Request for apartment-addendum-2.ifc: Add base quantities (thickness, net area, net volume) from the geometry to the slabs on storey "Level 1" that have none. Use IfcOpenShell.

First a look at what the model holds.

```python
import ifcopenshell
import ifcopenshell.util.element
import ifcopenshell.util.unit

model = ifcopenshell.open("apartment-addendum-2.ifc")
print(model.schema)
for unit_type in ("LENGTHUNIT", "AREAUNIT", "VOLUMEUNIT"):
    print(unit_type, ifcopenshell.util.unit.calculate_unit_scale(model, unit_type))
storey = next(s for s in model.by_type("IfcBuildingStorey") if s.Name == "Level 1")
slabs = [e for e in ifcopenshell.util.element.get_decomposition(storey) if e.is_a("IfcSlab")]
for e in sorted(slabs, key=lambda e: e.id()):
    print(e.id(), e.is_a(), e.Name, list(ifcopenshell.util.element.get_psets(e, qtos_only=True)), sep=" | ")
```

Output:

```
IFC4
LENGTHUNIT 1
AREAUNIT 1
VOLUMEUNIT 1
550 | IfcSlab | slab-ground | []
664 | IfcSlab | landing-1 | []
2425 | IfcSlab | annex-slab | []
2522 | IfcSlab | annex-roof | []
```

```python
import ifcopenshell
import ifcopenshell.api.pset
import ifcopenshell.geom
import ifcopenshell.util.element
import ifcopenshell.util.shape
import ifcopenshell.util.unit

model = ifcopenshell.open("apartment-addendum-2.ifc")
unit_scale = ifcopenshell.util.unit.calculate_unit_scale(model)
area_scale = ifcopenshell.util.unit.calculate_unit_scale(model, "AREAUNIT")
volume_scale = ifcopenshell.util.unit.calculate_unit_scale(model, "VOLUMEUNIT")
settings = ifcopenshell.geom.settings()

storey = next(s for s in model.by_type("IfcBuildingStorey") if s.Name == "Level 1")
slabs = [e for e in ifcopenshell.util.element.get_decomposition(storey) if e.is_a("IfcSlab")]

for e in sorted(slabs, key=lambda e: e.id()):
    if ifcopenshell.util.element.get_psets(e, qtos_only=True, should_inherit=False):
        continue
    # Geometry comes back in metres, in the element's own axes.
    shape = ifcopenshell.geom.create_shape(settings, e)
    values = {
        "Width": ifcopenshell.util.shape.get_z(shape.geometry) / unit_scale,
        "NetArea": ifcopenshell.util.shape.get_footprint_area(shape.geometry) / area_scale,
        "NetVolume": ifcopenshell.util.shape.get_volume(shape.geometry) / volume_scale,
    }
    qto = ifcopenshell.api.pset.add_qto(model, product=e, name="Qto_SlabBaseQuantities")
    ifcopenshell.api.pset.edit_qto(model, qto=qto, properties=values)
    print(e.id(), {k: round(v, 3) for k, v in values.items()})

model.write("apartment-addendum-2_rev.ifc")
```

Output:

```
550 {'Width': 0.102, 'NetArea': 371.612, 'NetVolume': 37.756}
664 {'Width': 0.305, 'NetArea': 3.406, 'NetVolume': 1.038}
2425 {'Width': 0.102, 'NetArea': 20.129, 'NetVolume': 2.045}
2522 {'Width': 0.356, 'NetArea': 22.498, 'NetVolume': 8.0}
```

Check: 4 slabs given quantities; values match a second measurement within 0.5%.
